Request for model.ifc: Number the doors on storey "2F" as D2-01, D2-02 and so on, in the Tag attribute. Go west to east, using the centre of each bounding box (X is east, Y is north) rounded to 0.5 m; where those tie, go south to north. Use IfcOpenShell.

First a look at what the model holds.

```python
import ifcopenshell
import ifcopenshell.util.element
import ifcopenshell.util.placement

model = ifcopenshell.open("model.ifc")
print(model.schema)
storey = next(s for s in model.by_type("IfcBuildingStorey") if s.Name == "2F")
doors = [e for e in ifcopenshell.util.element.get_decomposition(storey) if e.is_a("IfcDoor")]
for e in sorted(doors, key=lambda e: e.id()):
    origin = ifcopenshell.util.placement.get_local_placement(e.ObjectPlacement)[:3, 3]
    print(e.id(), e.Tag, e.Name, origin.round(2) + 0.0, sep=" | ")
```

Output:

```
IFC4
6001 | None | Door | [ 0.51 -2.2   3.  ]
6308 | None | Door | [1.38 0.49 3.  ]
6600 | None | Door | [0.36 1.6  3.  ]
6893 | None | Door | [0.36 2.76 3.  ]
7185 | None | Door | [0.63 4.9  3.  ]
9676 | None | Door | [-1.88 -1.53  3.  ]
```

```python
import ifcopenshell
import ifcopenshell.geom
import ifcopenshell.util.element
import ifcopenshell.util.shape

model = ifcopenshell.open("model.ifc")
settings = ifcopenshell.geom.settings()
settings.set("use-world-coords", True)


def centre(element):
    shape = ifcopenshell.geom.create_shape(settings, element)
    return ifcopenshell.util.shape.get_bbox_centroid(shape.geometry)


storey = next(s for s in model.by_type("IfcBuildingStorey") if s.Name == "2F")
doors = [e for e in ifcopenshell.util.element.get_decomposition(storey) if e.is_a("IfcDoor")]

# Insertion points can sit at a corner or the storey origin, so sort by the geometry (in metres).
centres = {e: centre(e) for e in doors}
doors.sort(key=lambda e: (round(centres[e][0] / 0.5), centres[e][1]))

for i, e in enumerate(doors, start=1):
    number = f"D2-{i:02d}"
    e.Tag = number
    print(e.id(), number)

model.write("model_updated.ifc")
```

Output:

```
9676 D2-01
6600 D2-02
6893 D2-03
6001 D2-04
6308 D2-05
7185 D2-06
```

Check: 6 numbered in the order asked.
